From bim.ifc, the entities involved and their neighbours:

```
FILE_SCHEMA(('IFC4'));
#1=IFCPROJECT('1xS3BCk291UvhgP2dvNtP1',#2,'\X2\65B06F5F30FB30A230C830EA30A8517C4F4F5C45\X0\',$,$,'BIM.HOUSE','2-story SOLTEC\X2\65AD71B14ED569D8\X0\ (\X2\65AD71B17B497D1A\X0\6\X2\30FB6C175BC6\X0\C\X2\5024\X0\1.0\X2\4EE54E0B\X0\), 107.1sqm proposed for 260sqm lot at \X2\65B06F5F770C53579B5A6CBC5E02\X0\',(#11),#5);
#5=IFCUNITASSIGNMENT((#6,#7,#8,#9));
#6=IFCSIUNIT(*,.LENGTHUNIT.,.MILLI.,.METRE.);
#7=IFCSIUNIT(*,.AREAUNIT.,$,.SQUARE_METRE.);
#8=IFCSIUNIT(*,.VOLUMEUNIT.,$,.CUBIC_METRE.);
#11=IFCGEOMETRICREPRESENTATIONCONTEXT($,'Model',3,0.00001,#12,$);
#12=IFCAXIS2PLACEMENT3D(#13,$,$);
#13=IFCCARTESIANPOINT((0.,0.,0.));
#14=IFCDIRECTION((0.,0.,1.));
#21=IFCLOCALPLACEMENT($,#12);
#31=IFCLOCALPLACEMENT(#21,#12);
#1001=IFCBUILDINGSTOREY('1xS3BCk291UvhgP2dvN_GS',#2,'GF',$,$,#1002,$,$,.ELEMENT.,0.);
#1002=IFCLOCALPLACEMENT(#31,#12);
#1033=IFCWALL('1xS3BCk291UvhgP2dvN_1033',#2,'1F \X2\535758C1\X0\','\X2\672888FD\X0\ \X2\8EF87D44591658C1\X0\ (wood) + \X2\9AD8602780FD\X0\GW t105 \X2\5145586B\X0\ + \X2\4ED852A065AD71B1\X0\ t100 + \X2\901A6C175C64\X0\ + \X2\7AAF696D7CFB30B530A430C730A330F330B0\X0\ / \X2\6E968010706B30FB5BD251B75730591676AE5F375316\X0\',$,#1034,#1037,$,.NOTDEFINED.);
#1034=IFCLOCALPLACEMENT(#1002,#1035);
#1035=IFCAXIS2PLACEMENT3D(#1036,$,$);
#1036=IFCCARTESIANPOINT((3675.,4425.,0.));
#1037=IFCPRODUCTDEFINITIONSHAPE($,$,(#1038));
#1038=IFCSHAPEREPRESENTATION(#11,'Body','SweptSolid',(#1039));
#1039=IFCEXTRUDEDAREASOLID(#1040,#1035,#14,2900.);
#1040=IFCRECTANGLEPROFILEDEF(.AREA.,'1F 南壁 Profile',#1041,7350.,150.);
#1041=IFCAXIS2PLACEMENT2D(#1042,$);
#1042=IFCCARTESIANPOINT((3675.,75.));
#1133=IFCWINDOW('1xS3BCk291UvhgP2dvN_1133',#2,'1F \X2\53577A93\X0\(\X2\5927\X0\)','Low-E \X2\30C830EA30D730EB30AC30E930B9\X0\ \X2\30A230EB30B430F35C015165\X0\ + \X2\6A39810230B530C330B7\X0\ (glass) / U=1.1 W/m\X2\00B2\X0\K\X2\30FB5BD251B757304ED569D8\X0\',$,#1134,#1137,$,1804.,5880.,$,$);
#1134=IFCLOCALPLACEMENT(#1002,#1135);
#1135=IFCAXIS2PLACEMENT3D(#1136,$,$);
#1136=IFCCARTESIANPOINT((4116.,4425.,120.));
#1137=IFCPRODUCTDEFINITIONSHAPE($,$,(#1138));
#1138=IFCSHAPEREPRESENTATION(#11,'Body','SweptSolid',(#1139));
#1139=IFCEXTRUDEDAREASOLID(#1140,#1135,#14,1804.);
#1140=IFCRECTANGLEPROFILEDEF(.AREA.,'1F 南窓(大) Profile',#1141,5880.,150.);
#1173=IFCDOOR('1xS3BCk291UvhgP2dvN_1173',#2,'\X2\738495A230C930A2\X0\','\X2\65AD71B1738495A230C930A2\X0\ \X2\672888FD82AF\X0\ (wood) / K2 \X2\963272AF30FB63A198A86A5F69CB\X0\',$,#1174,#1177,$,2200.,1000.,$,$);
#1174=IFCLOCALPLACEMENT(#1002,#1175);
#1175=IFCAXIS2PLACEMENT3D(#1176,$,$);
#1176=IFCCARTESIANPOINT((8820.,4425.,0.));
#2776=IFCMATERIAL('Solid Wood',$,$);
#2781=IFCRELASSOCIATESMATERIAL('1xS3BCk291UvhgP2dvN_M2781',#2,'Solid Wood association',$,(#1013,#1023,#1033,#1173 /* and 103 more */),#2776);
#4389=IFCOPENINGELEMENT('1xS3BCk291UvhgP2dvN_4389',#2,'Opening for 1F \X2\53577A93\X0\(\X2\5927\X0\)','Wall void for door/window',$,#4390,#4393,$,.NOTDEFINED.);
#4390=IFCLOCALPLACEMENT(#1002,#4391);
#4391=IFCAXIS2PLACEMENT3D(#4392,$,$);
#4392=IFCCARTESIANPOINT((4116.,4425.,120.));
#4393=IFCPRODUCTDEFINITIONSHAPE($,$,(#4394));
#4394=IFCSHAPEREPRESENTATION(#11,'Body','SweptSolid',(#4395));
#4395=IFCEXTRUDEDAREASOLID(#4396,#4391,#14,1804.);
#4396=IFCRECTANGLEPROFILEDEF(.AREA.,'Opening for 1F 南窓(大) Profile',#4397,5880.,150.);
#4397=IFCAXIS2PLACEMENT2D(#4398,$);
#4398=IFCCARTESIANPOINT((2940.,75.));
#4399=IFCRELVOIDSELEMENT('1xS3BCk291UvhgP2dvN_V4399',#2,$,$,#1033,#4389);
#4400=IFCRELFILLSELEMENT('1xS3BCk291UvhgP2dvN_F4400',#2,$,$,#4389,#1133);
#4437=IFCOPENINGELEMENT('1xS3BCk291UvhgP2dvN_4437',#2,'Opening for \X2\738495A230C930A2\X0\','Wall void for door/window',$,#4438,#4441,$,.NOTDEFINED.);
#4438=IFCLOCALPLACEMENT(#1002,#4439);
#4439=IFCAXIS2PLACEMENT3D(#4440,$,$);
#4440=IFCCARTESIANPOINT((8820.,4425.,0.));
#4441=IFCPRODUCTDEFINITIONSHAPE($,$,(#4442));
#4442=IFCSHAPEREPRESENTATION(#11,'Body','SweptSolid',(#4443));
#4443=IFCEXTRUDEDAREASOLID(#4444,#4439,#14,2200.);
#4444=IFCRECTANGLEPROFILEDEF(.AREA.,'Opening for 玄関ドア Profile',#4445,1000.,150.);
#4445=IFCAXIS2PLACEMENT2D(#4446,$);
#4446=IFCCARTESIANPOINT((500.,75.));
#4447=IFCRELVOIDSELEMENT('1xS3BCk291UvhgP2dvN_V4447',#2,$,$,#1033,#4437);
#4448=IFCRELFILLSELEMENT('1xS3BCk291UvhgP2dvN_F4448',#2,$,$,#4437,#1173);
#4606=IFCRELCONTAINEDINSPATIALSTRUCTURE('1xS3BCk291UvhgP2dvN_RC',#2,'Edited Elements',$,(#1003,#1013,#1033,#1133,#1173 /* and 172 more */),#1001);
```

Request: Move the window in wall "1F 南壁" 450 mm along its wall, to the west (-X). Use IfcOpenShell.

```python
import ifcopenshell
import ifcopenshell.api.geometry
import ifcopenshell.util.placement

model = ifcopenshell.open("bim.ifc")

window = model.by_guid("1xS3BCk291UvhgP2dvN_1133")
opening = window.FillsVoids[0].RelatingOpeningElement
wall = opening.VoidsElements[0].RelatingBuildingElement

wall_matrix = ifcopenshell.util.placement.get_local_placement(wall.ObjectPlacement)
shift = wall_matrix[:3, 0] * -450.0
before = ifcopenshell.util.placement.get_local_placement(window.ObjectPlacement)[:3, 3].copy()

# The window is not placed relative to its opening, so move both.
for product in (opening, window):
    matrix = ifcopenshell.util.placement.get_local_placement(product.ObjectPlacement)
    matrix[:3, 3] += shift
    ifcopenshell.api.geometry.edit_object_placement(model, product=product, matrix=matrix, is_si=False)

after = ifcopenshell.util.placement.get_local_placement(window.ObjectPlacement)[:3, 3]
print("window moved by", (after - before).round(3) + 0.0)

model.write("bim_updated.ifc")
```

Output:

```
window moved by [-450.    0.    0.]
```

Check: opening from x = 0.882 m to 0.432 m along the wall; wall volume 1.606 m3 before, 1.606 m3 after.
